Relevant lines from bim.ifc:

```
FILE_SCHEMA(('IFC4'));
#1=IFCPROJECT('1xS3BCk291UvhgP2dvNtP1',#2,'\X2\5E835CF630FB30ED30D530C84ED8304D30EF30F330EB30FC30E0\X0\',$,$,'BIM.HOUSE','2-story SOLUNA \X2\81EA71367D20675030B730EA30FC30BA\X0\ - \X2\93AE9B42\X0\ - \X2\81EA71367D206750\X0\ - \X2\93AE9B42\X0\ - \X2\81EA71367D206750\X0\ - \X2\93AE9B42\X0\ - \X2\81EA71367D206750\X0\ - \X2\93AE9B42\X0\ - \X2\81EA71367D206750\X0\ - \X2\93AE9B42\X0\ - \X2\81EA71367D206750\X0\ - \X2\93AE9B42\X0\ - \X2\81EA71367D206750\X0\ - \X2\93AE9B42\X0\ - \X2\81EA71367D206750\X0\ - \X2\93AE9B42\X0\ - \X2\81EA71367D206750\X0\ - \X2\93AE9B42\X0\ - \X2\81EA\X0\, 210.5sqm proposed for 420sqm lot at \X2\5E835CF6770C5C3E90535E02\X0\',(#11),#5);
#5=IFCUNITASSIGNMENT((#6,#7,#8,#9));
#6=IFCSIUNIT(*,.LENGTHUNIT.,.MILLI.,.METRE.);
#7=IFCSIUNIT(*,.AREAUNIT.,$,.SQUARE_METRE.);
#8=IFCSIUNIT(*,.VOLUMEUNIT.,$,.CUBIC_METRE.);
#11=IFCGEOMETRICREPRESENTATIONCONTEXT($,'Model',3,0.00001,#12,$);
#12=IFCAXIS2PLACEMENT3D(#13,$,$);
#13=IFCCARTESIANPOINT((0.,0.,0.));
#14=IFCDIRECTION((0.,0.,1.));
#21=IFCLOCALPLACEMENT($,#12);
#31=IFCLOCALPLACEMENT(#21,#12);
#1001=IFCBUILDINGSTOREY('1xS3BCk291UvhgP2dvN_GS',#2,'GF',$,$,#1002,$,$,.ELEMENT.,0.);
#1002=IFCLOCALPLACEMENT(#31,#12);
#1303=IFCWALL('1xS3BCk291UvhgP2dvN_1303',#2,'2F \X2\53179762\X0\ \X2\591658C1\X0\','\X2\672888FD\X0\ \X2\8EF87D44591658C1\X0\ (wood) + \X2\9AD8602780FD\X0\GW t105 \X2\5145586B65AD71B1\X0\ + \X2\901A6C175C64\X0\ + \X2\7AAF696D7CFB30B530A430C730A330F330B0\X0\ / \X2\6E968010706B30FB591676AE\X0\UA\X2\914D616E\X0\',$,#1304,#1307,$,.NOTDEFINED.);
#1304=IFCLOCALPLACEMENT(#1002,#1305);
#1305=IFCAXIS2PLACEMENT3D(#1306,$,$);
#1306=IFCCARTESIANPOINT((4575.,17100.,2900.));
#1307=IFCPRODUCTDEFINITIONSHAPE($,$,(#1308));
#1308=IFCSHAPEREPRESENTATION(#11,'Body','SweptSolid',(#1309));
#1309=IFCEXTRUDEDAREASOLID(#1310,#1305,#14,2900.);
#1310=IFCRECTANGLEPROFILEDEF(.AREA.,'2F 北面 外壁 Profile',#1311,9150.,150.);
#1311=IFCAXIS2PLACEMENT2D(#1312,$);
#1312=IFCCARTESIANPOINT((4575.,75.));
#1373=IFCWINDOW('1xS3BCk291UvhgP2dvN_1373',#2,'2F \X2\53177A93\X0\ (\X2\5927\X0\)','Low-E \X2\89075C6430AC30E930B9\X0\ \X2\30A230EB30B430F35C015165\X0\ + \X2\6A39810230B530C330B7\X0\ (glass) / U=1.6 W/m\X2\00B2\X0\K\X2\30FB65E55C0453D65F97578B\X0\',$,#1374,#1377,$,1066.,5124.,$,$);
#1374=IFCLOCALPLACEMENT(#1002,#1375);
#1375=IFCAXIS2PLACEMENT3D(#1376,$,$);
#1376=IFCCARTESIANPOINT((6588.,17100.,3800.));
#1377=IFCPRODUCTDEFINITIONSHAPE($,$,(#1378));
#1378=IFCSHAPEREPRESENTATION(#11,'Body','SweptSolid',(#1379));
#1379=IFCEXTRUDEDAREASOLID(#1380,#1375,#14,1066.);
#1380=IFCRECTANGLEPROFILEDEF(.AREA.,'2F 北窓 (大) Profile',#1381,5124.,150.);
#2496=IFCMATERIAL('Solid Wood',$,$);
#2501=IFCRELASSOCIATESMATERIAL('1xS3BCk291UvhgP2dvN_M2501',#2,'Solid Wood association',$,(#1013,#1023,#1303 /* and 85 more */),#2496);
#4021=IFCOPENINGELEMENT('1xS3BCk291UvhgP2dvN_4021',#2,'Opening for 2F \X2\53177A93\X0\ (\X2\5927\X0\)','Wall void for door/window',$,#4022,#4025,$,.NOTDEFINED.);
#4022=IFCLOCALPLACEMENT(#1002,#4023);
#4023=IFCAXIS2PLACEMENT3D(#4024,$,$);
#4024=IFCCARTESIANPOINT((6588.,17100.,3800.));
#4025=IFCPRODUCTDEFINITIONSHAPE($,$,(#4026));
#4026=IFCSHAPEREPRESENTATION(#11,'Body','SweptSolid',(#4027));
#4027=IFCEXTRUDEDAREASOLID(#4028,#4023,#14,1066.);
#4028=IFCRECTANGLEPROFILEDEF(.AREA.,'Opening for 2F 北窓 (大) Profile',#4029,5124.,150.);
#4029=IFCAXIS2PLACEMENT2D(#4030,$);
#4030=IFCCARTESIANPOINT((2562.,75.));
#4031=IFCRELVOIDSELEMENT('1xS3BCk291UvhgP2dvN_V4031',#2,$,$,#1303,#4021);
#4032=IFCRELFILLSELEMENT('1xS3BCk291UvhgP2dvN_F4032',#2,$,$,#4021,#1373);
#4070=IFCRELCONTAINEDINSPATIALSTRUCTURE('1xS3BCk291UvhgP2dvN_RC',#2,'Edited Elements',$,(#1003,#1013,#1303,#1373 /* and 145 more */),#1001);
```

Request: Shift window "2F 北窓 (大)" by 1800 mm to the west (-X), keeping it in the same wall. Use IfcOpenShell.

```python
import ifcopenshell
import ifcopenshell.api.geometry
import ifcopenshell.util.placement
import ifcopenshell.util.unit

model = ifcopenshell.open("bim.ifc")
unit_scale = ifcopenshell.util.unit.calculate_unit_scale(model)

window = model.by_id(1373)
opening = window.FillsVoids[0].RelatingOpeningElement
wall = opening.VoidsElements[0].RelatingBuildingElement

wall_matrix = ifcopenshell.util.placement.get_local_placement(wall.ObjectPlacement)
shift = wall_matrix[:3, 0] * -1.8 / unit_scale
before = ifcopenshell.util.placement.get_local_placement(window.ObjectPlacement)[:3, 3].copy()

# The window is not placed relative to its opening, so move both.
for product in (opening, window):
    matrix = ifcopenshell.util.placement.get_local_placement(product.ObjectPlacement)
    matrix[:3, 3] += shift
    ifcopenshell.api.geometry.edit_object_placement(model, product=product, matrix=matrix, is_si=False)

after = ifcopenshell.util.placement.get_local_placement(window.ObjectPlacement)[:3, 3]
print("window moved by", (after - before).round(3) + 0.0)

model.write("bim_edited.ifc")
```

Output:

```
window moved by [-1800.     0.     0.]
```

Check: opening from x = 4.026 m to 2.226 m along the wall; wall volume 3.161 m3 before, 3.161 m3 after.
